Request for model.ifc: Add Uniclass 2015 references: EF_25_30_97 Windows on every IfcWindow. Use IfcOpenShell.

First a look at what the model holds.

```python
import ifcopenshell

model = ifcopenshell.open("model.ifc")
print(model.schema)
print("classifications:", [c.Name for c in model.by_type("IfcClassification")])
for ifc_class in ("IfcDoor", "IfcRoof", "IfcStair", "IfcWall", "IfcWindow"):
    print(ifc_class, len(model.by_type(ifc_class)))
```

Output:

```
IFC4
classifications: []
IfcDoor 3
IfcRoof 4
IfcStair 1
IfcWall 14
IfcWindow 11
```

```python
import ifcopenshell
import ifcopenshell.api.classification

model = ifcopenshell.open("model.ifc")

system = ifcopenshell.api.classification.add_classification(model, classification="Uniclass 2015")

codes = {
    "IfcWindow": ("EF_25_30_97", "Windows"),
}
for ifc_class, (code, name) in codes.items():
    products = model.by_type(ifc_class)
    ifcopenshell.api.classification.add_reference(
        model, products=products, classification=system, identification=code, name=name
    )
    print(code, len(products))

model.write("model_edited.ifc")
```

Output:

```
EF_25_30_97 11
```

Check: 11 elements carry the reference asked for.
